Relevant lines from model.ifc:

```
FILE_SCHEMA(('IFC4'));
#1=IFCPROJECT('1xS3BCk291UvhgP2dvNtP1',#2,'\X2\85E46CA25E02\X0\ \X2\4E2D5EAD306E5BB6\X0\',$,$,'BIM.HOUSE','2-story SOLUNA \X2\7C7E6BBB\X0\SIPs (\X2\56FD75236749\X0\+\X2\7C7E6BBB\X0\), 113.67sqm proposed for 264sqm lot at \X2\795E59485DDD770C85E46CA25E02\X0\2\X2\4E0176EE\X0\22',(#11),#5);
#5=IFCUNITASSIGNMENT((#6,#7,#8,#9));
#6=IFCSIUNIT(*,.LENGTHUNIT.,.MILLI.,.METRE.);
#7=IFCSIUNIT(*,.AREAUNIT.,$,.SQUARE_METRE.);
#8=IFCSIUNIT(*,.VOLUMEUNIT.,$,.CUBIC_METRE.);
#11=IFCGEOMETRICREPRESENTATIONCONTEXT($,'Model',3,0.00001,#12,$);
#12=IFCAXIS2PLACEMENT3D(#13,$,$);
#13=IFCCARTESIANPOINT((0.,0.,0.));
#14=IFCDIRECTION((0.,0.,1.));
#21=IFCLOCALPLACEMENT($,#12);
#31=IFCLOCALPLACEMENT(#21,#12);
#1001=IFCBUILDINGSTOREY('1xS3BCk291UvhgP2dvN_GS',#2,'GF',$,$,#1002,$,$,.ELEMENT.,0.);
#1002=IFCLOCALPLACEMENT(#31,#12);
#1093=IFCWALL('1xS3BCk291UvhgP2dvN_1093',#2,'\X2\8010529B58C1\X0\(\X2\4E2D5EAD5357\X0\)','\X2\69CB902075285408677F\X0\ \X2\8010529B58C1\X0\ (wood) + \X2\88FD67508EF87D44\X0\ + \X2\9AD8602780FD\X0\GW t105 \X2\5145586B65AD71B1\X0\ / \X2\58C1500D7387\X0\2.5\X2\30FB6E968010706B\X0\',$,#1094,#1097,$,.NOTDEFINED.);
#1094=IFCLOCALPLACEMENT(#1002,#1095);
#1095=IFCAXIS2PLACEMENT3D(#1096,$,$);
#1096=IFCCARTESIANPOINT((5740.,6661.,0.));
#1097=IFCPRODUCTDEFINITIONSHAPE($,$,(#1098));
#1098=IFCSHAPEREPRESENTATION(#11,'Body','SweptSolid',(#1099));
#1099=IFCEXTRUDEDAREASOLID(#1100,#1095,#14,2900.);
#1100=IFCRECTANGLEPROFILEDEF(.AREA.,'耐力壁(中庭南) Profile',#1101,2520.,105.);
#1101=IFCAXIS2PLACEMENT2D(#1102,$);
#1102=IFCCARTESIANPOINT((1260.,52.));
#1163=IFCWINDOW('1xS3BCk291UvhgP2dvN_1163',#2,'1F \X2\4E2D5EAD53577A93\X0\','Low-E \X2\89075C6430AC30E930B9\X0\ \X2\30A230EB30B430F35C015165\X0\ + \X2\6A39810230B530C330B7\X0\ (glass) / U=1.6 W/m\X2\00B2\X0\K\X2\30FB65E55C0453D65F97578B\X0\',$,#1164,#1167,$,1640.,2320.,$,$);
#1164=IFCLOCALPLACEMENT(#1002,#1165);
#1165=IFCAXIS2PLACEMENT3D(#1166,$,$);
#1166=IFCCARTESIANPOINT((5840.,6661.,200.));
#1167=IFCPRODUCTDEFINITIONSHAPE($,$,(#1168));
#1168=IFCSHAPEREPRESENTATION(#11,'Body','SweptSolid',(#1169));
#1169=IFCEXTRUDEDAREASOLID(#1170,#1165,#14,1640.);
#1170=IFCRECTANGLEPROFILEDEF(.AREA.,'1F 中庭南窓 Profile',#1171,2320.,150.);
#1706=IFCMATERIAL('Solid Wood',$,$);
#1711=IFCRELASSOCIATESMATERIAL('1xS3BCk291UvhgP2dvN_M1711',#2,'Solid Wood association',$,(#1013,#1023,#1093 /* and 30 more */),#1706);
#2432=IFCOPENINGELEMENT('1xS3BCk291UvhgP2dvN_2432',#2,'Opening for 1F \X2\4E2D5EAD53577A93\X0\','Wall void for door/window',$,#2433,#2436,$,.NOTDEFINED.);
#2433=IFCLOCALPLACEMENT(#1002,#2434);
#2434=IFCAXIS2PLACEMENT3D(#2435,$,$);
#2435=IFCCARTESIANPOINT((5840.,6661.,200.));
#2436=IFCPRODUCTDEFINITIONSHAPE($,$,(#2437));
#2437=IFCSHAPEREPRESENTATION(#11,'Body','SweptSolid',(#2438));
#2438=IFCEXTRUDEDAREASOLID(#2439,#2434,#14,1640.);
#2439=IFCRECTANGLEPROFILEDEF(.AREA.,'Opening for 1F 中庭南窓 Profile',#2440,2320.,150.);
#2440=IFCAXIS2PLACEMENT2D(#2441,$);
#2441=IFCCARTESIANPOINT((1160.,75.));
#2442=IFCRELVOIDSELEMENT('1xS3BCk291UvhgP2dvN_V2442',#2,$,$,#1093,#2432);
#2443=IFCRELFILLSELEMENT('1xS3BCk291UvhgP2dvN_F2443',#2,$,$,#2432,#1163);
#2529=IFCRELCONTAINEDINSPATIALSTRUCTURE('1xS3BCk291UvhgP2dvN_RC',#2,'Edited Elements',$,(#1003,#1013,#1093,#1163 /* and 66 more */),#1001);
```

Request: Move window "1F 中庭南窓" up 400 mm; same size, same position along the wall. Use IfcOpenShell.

```python
import numpy as np
import ifcopenshell
import ifcopenshell.api.geometry
import ifcopenshell.util.placement
import ifcopenshell.util.unit

model = ifcopenshell.open("model.ifc")
unit_scale = ifcopenshell.util.unit.calculate_unit_scale(model)

window = model.by_guid("1xS3BCk291UvhgP2dvN_1163")
opening = window.FillsVoids[0].RelatingOpeningElement
dz = 0.4 / unit_scale

shift = np.array([0.0, 0.0, dz])
# The window is not placed relative to its opening, so move both.
for product in (opening, window):
    matrix = ifcopenshell.util.placement.get_local_placement(product.ObjectPlacement)
    matrix[:3, 3] += shift
    ifcopenshell.api.geometry.edit_object_placement(model, product=product, matrix=matrix, is_si=False)

print(f"moved by {dz * unit_scale:+.3f} m")

model.write("model_rev.ifc")
```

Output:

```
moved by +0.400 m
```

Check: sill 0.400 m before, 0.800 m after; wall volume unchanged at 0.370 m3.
